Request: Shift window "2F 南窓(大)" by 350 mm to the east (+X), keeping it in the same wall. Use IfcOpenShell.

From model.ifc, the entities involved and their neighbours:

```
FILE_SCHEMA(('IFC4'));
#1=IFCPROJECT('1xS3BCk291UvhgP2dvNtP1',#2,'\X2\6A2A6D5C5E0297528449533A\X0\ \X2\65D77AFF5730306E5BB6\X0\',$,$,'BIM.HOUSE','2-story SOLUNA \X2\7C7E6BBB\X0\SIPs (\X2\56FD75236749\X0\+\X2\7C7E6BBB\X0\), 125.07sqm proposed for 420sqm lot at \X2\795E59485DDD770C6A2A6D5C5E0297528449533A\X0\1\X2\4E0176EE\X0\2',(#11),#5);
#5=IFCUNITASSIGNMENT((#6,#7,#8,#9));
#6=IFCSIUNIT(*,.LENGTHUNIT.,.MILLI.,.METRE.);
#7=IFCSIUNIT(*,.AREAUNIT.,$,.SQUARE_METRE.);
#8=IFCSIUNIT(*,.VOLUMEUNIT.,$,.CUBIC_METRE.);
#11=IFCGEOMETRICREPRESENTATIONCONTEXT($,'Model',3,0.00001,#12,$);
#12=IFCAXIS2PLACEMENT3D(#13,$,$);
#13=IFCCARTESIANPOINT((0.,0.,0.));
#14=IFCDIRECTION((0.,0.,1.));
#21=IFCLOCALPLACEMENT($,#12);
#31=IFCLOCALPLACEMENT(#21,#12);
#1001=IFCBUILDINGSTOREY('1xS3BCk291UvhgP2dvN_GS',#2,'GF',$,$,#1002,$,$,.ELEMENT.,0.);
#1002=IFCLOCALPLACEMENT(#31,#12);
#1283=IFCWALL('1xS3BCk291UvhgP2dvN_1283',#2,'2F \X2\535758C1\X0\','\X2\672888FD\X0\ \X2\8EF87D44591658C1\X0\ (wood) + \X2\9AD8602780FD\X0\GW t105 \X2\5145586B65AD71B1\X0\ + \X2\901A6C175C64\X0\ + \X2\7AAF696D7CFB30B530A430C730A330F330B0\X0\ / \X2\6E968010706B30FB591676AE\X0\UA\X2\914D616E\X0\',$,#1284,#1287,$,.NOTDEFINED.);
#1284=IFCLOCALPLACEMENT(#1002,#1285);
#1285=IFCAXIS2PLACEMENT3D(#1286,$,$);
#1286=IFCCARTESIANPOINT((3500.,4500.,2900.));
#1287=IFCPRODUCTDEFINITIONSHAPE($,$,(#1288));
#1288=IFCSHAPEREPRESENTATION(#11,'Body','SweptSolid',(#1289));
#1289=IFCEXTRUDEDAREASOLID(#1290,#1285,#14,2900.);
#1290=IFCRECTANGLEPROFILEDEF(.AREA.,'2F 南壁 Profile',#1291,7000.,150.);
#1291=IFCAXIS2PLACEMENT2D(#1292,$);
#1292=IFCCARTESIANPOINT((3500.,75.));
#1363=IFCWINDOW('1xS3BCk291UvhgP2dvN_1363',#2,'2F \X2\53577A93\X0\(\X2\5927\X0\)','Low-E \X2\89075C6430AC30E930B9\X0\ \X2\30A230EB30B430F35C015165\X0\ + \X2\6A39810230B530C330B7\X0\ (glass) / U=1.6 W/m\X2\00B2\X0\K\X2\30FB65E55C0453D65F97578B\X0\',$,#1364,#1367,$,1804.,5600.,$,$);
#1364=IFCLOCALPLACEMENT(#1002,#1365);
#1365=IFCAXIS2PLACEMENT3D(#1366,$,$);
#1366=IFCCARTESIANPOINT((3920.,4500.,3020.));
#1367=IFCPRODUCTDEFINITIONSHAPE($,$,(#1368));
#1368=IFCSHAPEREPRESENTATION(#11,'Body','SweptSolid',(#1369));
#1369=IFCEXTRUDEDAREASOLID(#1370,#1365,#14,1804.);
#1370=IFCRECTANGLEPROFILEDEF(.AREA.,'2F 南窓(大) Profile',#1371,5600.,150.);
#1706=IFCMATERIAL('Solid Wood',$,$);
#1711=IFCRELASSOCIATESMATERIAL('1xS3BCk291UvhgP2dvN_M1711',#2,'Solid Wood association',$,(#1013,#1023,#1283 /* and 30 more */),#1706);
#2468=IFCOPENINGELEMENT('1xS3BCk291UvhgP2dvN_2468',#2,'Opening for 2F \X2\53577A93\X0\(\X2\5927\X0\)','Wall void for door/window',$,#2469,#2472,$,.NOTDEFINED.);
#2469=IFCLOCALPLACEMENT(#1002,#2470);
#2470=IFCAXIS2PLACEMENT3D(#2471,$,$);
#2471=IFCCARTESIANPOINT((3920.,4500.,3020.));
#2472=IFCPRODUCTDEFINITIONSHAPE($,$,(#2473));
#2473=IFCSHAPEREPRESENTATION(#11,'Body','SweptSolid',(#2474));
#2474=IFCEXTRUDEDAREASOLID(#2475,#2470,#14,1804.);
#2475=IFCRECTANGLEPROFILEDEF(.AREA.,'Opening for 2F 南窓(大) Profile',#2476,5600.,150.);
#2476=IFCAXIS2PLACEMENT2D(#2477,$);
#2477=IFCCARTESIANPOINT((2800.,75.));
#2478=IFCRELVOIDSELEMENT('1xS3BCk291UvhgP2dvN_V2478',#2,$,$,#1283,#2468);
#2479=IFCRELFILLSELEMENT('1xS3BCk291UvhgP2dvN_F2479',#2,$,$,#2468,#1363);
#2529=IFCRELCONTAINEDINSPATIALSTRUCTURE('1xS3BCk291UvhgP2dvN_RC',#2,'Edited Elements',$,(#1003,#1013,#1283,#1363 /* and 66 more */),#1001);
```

```python
import ifcopenshell
import ifcopenshell.api.geometry
import ifcopenshell.util.placement

model = ifcopenshell.open("model.ifc")

window = model.by_guid("1xS3BCk291UvhgP2dvN_1363")
opening = window.FillsVoids[0].RelatingOpeningElement
wall = opening.VoidsElements[0].RelatingBuildingElement

wall_matrix = ifcopenshell.util.placement.get_local_placement(wall.ObjectPlacement)
shift = wall_matrix[:3, 0] * 350.0
before = ifcopenshell.util.placement.get_local_placement(window.ObjectPlacement)[:3, 3].copy()

# The window is not placed relative to its opening, so move both.
for product in (opening, window):
    matrix = ifcopenshell.util.placement.get_local_placement(product.ObjectPlacement)
    matrix[:3, 3] += shift
    ifcopenshell.api.geometry.edit_object_placement(model, product=product, matrix=matrix, is_si=False)

after = ifcopenshell.util.placement.get_local_placement(window.ObjectPlacement)[:3, 3]
print("window moved by", (after - before).round(3) + 0.0)

model.write("model_edited.ifc")
```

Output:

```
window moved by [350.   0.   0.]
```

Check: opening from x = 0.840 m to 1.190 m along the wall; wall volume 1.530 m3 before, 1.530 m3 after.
